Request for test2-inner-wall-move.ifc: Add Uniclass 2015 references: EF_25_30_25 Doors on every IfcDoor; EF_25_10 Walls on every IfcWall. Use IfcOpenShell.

First a look at what the model holds.

```python
import ifcopenshell

model = ifcopenshell.open("test2-inner-wall-move.ifc")
print(model.schema)
print("classifications:", [c.Name for c in model.by_type("IfcClassification")])
for ifc_class in ("IfcDoor", "IfcRoof", "IfcStair", "IfcWall", "IfcWindow"):
    print(ifc_class, len(model.by_type(ifc_class)))
```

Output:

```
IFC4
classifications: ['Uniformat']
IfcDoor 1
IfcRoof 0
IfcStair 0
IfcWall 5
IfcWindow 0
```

```python
import ifcopenshell
import ifcopenshell.api.classification

model = ifcopenshell.open("test2-inner-wall-move.ifc")

system = ifcopenshell.api.classification.add_classification(model, classification="Uniclass 2015")

codes = {
    "IfcDoor": ("EF_25_30_25", "Doors"),
    "IfcWall": ("EF_25_10", "Walls"),
}
for ifc_class, (code, name) in codes.items():
    products = model.by_type(ifc_class)
    ifcopenshell.api.classification.add_reference(
        model, products=products, classification=system, identification=code, name=name
    )
    print(code, len(products))

model.write("test2-inner-wall-move_rev.ifc")
```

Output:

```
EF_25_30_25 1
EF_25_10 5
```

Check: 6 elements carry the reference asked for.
